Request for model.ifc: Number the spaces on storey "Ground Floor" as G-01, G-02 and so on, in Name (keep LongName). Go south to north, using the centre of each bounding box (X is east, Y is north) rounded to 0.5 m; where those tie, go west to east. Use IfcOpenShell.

First a look at what the model holds.

```python
import ifcopenshell
import ifcopenshell.util.element
import ifcopenshell.util.placement

model = ifcopenshell.open("model.ifc")
print(model.schema)
storey = next(s for s in model.by_type("IfcBuildingStorey") if s.Name == "Ground Floor")
spaces = [e for e in ifcopenshell.util.element.get_decomposition(storey) if e.is_a("IfcSpace")]
for e in sorted(spaces, key=lambda e: e.id()):
    origin = ifcopenshell.util.placement.get_local_placement(e.ObjectPlacement)[:3, 3]
    print(e.id(), e.Name, e.LongName, origin.round(2) + 0.0, sep=" | ")
```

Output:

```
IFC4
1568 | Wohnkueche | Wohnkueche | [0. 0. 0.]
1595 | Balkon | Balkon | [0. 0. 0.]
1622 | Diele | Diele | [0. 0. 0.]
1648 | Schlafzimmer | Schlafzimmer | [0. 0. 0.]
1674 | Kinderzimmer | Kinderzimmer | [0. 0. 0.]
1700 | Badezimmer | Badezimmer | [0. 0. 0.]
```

```python
import ifcopenshell
import ifcopenshell.geom
import ifcopenshell.util.element
import ifcopenshell.util.shape

model = ifcopenshell.open("model.ifc")
settings = ifcopenshell.geom.settings()
settings.set("use-world-coords", True)


def centre(element):
    shape = ifcopenshell.geom.create_shape(settings, element)
    return ifcopenshell.util.shape.get_bbox_centroid(shape.geometry)


storey = next(s for s in model.by_type("IfcBuildingStorey") if s.Name == "Ground Floor")
spaces = [e for e in ifcopenshell.util.element.get_decomposition(storey) if e.is_a("IfcSpace")]

# Insertion points can sit at a corner or the storey origin, so sort by the geometry (in metres).
centres = {e: centre(e) for e in spaces}
spaces.sort(key=lambda e: (round(centres[e][1] / 0.5), centres[e][0]))

for i, e in enumerate(spaces, start=1):
    number = f"G-{i:02d}"
    e.Name = number
    print(e.id(), number)

model.write("model-out.ifc")
```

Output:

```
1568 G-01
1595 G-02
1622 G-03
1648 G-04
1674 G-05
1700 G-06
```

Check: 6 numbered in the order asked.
